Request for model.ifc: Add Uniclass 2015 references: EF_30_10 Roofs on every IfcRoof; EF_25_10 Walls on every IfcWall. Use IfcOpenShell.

First a look at what the model holds.

```python
import ifcopenshell

model = ifcopenshell.open("model.ifc")
print(model.schema)
print("classifications:", [c.Name for c in model.by_type("IfcClassification")])
for ifc_class in ("IfcDoor", "IfcRoof", "IfcStair", "IfcWall", "IfcWindow"):
    print(ifc_class, len(model.by_type(ifc_class)))
```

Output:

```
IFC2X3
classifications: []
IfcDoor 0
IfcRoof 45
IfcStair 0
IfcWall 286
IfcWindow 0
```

```python
import ifcopenshell
import ifcopenshell.api.classification

model = ifcopenshell.open("model.ifc")

# IFC2X3 requires Source and Edition and has no link from the project to the system.
system = model.create_entity("IfcClassification", Source="NBS", Edition="2015", Name="Uniclass 2015")

codes = {
    "IfcRoof": ("EF_30_10", "Roofs"),
    "IfcWall": ("EF_25_10", "Walls"),
}
for ifc_class, (code, name) in codes.items():
    products = model.by_type(ifc_class)
    ifcopenshell.api.classification.add_reference(
        model, products=products, classification=system, identification=code, name=name
    )
    print(code, len(products))

model.write("model-out.ifc")
```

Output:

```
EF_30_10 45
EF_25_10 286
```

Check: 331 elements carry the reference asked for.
